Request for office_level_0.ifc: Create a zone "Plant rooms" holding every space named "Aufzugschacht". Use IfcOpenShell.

First a look at what the model holds.

```python
import ifcopenshell

model = ifcopenshell.open("office_level_0.ifc")
print(model.schema)
seen = {}
for space in model.by_type("IfcSpace"):
    seen[space.LongName] = seen.get(space.LongName, 0) + 1
for name, count in sorted(seen.items(), key=str):
    print(count, "x", name)
print("zones:", [z.Name for z in model.by_type("IfcZone")][:20])
```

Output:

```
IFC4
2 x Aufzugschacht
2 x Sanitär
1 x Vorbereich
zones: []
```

```python
import ifcopenshell
import ifcopenshell.api.group
import ifcopenshell.api.root

model = ifcopenshell.open("office_level_0.ifc")

names = {"Aufzugschacht"}
spaces = [s for s in model.by_type("IfcSpace") if s.LongName in names]

zone = ifcopenshell.api.root.create_entity(model, ifc_class="IfcZone", name="Plant rooms")
ifcopenshell.api.group.assign_group(model, products=spaces, group=zone)
print(len(spaces), "spaces in", zone.Name)

model.write("office_level_0_rev.ifc")
```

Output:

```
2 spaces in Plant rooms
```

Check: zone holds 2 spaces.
